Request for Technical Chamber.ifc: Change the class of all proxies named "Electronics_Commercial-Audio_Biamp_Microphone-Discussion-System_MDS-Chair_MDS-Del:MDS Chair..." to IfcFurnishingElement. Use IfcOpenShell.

First a look at what the model holds.

```python
import re

import ifcopenshell

model = ifcopenshell.open("Technical Chamber.ifc")
print(model.schema)
seen = {}
for e in model.by_type("IfcBuildingElementProxy"):
    name = re.sub(r":\d+(:\d+)?$", "", e.Name or "")  # drop the element id that some exporters append
    seen[name] = seen.get(name, 0) + 1
for name, count in sorted(seen.items()):
    print(count, "x", name)
```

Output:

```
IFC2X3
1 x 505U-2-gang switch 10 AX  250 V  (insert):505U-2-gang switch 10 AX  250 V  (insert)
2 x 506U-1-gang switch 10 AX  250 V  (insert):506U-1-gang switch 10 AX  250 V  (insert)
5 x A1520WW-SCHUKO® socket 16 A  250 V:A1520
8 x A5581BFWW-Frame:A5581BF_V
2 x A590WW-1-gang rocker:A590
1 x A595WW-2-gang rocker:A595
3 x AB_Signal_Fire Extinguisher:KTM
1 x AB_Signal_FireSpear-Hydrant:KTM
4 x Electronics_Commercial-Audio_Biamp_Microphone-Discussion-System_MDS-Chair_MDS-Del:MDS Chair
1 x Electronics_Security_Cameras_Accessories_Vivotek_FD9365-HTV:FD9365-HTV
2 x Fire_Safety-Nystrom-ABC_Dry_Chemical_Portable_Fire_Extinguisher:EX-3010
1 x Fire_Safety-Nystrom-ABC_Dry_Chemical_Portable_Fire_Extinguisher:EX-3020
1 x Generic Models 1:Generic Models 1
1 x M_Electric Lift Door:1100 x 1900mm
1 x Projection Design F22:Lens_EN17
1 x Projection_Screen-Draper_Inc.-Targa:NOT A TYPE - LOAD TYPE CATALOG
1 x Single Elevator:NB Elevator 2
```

```python
import ifcopenshell
import ifcopenshell.api.root

model = ifcopenshell.open("Technical Chamber.ifc")

proxies = [e.id() for e in model.by_type("IfcBuildingElementProxy") if (e.Name or "").startswith("Electronics_Commercial-Audio_Biamp_Microphone-Discussion-System_MDS-Chair_MDS-Del:MDS Chair")]
for step_id in proxies:
    proxy = model.by_id(step_id)
    # Reclassifying a typed element also reclassifies its type and the type's other occurrences.
    if proxy.is_a("IfcBuildingElementProxy"):
        ifcopenshell.api.root.reassign_class(model, product=proxy, ifc_class="IfcFurnishingElement")

print(sum(model.by_id(i).is_a("IfcFurnishingElement") for i in proxies), "reclassified")

model.write("Technical Chamber_updated.ifc")
```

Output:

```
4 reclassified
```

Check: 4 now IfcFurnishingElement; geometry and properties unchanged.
